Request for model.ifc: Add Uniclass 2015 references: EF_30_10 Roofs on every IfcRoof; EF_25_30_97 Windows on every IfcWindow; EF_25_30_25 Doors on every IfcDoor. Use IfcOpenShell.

First a look at what the model holds.

```python
import ifcopenshell

model = ifcopenshell.open("model.ifc")
print(model.schema)
print("classifications:", [c.Name for c in model.by_type("IfcClassification")])
for ifc_class in ("IfcDoor", "IfcRoof", "IfcStair", "IfcWall", "IfcWindow"):
    print(ifc_class, len(model.by_type(ifc_class)))
```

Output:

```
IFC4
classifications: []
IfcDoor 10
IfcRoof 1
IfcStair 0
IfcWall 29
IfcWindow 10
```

```python
import ifcopenshell
import ifcopenshell.api.classification

model = ifcopenshell.open("model.ifc")

system = ifcopenshell.api.classification.add_classification(model, classification="Uniclass 2015")

codes = {
    "IfcRoof": ("EF_30_10", "Roofs"),
    "IfcWindow": ("EF_25_30_97", "Windows"),
    "IfcDoor": ("EF_25_30_25", "Doors"),
}
for ifc_class, (code, name) in codes.items():
    products = model.by_type(ifc_class)
    ifcopenshell.api.classification.add_reference(
        model, products=products, classification=system, identification=code, name=name
    )
    print(code, len(products))

model.write("model_rev.ifc")
```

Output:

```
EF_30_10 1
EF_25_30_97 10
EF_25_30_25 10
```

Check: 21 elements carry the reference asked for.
